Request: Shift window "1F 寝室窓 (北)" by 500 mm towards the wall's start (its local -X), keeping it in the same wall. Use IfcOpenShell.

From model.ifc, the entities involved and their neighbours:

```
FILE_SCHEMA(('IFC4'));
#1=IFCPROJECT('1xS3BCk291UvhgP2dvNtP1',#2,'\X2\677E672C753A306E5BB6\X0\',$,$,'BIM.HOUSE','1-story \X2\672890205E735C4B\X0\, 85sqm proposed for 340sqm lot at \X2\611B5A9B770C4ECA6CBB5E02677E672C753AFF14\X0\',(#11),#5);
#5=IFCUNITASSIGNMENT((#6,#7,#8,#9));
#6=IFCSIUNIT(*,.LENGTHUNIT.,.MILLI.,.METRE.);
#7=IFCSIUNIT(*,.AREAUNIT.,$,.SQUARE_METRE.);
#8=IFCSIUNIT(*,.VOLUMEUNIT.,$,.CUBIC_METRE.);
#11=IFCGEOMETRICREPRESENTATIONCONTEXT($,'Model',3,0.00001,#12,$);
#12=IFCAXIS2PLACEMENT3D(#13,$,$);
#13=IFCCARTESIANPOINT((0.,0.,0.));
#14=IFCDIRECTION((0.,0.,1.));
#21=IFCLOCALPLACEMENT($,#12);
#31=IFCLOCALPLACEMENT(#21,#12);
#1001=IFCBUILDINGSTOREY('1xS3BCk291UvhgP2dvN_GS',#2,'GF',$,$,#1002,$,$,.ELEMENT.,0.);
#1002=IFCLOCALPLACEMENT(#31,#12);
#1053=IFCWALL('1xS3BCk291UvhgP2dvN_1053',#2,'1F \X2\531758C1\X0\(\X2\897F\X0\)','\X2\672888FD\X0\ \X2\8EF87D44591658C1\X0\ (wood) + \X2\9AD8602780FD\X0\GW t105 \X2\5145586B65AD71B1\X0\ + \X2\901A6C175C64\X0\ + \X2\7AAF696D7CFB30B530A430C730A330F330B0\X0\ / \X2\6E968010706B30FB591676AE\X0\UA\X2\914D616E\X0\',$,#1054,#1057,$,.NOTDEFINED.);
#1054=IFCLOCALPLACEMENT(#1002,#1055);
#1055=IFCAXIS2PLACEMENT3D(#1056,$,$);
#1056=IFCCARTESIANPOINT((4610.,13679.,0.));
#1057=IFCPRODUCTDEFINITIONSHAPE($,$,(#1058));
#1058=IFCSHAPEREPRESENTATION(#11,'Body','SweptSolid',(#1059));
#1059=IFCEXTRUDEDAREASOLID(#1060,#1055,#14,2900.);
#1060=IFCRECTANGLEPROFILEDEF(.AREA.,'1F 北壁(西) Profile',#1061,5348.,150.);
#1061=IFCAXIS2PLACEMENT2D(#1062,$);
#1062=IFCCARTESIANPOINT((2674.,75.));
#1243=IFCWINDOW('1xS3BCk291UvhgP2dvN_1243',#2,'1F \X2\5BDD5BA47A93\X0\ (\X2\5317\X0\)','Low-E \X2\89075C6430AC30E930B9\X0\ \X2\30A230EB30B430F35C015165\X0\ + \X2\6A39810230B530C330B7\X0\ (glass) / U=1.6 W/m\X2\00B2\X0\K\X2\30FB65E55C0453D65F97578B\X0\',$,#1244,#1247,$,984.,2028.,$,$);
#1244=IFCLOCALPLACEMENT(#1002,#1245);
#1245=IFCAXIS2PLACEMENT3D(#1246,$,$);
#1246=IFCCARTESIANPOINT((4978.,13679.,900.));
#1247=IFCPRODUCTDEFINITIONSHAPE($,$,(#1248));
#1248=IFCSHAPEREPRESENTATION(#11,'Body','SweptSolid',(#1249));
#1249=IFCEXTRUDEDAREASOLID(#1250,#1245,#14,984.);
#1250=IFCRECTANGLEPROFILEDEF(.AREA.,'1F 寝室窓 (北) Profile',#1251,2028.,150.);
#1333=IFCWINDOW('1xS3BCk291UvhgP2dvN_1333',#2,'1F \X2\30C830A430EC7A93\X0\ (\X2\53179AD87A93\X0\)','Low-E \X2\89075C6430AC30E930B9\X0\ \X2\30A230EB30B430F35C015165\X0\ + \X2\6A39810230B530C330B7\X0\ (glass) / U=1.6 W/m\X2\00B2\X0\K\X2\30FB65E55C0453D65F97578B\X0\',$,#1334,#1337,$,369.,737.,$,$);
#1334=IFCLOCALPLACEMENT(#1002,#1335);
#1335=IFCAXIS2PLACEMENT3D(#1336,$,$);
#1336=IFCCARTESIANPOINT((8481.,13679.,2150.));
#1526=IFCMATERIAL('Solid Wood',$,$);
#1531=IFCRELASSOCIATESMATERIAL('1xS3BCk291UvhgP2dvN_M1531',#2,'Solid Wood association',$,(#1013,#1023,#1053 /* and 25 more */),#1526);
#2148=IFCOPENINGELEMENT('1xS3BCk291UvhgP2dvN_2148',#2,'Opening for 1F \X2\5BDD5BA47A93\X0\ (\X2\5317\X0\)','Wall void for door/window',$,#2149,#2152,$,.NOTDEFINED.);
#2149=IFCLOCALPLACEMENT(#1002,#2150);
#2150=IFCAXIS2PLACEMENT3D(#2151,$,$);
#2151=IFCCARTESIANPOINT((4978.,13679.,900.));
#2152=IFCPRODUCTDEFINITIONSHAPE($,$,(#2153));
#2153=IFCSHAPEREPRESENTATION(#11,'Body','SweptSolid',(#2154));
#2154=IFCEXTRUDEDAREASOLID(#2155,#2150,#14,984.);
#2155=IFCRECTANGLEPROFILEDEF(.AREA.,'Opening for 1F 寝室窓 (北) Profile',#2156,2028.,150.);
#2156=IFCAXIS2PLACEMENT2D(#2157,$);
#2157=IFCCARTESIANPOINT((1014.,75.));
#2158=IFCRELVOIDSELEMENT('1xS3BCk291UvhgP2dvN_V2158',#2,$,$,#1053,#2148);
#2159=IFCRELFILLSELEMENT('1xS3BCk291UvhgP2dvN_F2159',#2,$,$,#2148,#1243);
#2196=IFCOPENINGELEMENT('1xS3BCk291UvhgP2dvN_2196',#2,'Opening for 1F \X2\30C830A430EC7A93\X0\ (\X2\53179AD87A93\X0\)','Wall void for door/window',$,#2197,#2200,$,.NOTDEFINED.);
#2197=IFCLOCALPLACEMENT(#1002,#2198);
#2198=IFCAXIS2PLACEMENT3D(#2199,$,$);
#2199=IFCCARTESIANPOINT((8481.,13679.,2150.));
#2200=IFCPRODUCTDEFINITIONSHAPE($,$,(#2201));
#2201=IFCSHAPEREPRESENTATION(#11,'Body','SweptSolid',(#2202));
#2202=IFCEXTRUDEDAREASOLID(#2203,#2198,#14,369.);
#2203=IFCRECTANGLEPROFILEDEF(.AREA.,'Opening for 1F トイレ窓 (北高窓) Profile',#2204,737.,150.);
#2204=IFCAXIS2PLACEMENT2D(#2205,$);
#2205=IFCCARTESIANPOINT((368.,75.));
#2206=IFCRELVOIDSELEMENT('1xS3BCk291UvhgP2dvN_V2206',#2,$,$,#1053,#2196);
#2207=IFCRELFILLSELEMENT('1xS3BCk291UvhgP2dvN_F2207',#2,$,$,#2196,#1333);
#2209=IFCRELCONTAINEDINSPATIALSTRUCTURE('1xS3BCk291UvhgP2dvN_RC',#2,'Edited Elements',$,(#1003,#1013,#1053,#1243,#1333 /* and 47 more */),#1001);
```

```python
import ifcopenshell
import ifcopenshell.api.geometry
import ifcopenshell.util.placement
import ifcopenshell.util.unit

model = ifcopenshell.open("model.ifc")
unit_scale = ifcopenshell.util.unit.calculate_unit_scale(model)

window = model.by_id(1243)
opening = window.FillsVoids[0].RelatingOpeningElement
wall = opening.VoidsElements[0].RelatingBuildingElement

wall_matrix = ifcopenshell.util.placement.get_local_placement(wall.ObjectPlacement)
shift = wall_matrix[:3, 0] * -0.5 / unit_scale
before = ifcopenshell.util.placement.get_local_placement(window.ObjectPlacement)[:3, 3].copy()

# The window is not placed relative to its opening, so move both.
for product in (opening, window):
    matrix = ifcopenshell.util.placement.get_local_placement(product.ObjectPlacement)
    matrix[:3, 3] += shift
    ifcopenshell.api.geometry.edit_object_placement(model, product=product, matrix=matrix, is_si=False)

after = ifcopenshell.util.placement.get_local_placement(window.ObjectPlacement)[:3, 3]
print("window moved by", (after - before).round(3) + 0.0)

model.write("model-out.ifc")
```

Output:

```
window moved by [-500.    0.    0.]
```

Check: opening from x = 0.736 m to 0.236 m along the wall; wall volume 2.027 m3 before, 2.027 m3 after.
